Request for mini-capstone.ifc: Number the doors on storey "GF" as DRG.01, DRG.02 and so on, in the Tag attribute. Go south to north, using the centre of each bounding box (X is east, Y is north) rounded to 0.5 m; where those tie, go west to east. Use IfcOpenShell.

First a look at what the model holds.

```python
import ifcopenshell
import ifcopenshell.util.element
import ifcopenshell.util.placement

model = ifcopenshell.open("mini-capstone.ifc")
print(model.schema)
storey = next(s for s in model.by_type("IfcBuildingStorey") if s.Name == "GF")
doors = [e for e in ifcopenshell.util.element.get_decomposition(storey) if e.is_a("IfcDoor")]
for e in sorted(doors, key=lambda e: e.id()):
    origin = ifcopenshell.util.placement.get_local_placement(e.ObjectPlacement)[:3, 3]
    print(e.id(), e.Tag, e.Name, origin.round(2) + 0.0, sep=" | ")
```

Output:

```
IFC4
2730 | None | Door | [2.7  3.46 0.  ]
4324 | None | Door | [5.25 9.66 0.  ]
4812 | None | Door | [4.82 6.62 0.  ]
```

```python
import ifcopenshell
import ifcopenshell.geom
import ifcopenshell.util.element
import ifcopenshell.util.shape

model = ifcopenshell.open("mini-capstone.ifc")
settings = ifcopenshell.geom.settings()
settings.set("use-world-coords", True)


def centre(element):
    shape = ifcopenshell.geom.create_shape(settings, element)
    return ifcopenshell.util.shape.get_bbox_centroid(shape.geometry)


storey = next(s for s in model.by_type("IfcBuildingStorey") if s.Name == "GF")
doors = [e for e in ifcopenshell.util.element.get_decomposition(storey) if e.is_a("IfcDoor")]

# Insertion points can sit at a corner or the storey origin, so sort by the geometry (in metres).
centres = {e: centre(e) for e in doors}
doors.sort(key=lambda e: (round(centres[e][1] / 0.5), centres[e][0]))

for i, e in enumerate(doors, start=1):
    number = f"DRG.{i:02d}"
    e.Tag = number
    print(e.id(), number)

model.write("mini-capstone_rev.ifc")
```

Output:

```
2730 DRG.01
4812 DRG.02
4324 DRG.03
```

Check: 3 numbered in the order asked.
